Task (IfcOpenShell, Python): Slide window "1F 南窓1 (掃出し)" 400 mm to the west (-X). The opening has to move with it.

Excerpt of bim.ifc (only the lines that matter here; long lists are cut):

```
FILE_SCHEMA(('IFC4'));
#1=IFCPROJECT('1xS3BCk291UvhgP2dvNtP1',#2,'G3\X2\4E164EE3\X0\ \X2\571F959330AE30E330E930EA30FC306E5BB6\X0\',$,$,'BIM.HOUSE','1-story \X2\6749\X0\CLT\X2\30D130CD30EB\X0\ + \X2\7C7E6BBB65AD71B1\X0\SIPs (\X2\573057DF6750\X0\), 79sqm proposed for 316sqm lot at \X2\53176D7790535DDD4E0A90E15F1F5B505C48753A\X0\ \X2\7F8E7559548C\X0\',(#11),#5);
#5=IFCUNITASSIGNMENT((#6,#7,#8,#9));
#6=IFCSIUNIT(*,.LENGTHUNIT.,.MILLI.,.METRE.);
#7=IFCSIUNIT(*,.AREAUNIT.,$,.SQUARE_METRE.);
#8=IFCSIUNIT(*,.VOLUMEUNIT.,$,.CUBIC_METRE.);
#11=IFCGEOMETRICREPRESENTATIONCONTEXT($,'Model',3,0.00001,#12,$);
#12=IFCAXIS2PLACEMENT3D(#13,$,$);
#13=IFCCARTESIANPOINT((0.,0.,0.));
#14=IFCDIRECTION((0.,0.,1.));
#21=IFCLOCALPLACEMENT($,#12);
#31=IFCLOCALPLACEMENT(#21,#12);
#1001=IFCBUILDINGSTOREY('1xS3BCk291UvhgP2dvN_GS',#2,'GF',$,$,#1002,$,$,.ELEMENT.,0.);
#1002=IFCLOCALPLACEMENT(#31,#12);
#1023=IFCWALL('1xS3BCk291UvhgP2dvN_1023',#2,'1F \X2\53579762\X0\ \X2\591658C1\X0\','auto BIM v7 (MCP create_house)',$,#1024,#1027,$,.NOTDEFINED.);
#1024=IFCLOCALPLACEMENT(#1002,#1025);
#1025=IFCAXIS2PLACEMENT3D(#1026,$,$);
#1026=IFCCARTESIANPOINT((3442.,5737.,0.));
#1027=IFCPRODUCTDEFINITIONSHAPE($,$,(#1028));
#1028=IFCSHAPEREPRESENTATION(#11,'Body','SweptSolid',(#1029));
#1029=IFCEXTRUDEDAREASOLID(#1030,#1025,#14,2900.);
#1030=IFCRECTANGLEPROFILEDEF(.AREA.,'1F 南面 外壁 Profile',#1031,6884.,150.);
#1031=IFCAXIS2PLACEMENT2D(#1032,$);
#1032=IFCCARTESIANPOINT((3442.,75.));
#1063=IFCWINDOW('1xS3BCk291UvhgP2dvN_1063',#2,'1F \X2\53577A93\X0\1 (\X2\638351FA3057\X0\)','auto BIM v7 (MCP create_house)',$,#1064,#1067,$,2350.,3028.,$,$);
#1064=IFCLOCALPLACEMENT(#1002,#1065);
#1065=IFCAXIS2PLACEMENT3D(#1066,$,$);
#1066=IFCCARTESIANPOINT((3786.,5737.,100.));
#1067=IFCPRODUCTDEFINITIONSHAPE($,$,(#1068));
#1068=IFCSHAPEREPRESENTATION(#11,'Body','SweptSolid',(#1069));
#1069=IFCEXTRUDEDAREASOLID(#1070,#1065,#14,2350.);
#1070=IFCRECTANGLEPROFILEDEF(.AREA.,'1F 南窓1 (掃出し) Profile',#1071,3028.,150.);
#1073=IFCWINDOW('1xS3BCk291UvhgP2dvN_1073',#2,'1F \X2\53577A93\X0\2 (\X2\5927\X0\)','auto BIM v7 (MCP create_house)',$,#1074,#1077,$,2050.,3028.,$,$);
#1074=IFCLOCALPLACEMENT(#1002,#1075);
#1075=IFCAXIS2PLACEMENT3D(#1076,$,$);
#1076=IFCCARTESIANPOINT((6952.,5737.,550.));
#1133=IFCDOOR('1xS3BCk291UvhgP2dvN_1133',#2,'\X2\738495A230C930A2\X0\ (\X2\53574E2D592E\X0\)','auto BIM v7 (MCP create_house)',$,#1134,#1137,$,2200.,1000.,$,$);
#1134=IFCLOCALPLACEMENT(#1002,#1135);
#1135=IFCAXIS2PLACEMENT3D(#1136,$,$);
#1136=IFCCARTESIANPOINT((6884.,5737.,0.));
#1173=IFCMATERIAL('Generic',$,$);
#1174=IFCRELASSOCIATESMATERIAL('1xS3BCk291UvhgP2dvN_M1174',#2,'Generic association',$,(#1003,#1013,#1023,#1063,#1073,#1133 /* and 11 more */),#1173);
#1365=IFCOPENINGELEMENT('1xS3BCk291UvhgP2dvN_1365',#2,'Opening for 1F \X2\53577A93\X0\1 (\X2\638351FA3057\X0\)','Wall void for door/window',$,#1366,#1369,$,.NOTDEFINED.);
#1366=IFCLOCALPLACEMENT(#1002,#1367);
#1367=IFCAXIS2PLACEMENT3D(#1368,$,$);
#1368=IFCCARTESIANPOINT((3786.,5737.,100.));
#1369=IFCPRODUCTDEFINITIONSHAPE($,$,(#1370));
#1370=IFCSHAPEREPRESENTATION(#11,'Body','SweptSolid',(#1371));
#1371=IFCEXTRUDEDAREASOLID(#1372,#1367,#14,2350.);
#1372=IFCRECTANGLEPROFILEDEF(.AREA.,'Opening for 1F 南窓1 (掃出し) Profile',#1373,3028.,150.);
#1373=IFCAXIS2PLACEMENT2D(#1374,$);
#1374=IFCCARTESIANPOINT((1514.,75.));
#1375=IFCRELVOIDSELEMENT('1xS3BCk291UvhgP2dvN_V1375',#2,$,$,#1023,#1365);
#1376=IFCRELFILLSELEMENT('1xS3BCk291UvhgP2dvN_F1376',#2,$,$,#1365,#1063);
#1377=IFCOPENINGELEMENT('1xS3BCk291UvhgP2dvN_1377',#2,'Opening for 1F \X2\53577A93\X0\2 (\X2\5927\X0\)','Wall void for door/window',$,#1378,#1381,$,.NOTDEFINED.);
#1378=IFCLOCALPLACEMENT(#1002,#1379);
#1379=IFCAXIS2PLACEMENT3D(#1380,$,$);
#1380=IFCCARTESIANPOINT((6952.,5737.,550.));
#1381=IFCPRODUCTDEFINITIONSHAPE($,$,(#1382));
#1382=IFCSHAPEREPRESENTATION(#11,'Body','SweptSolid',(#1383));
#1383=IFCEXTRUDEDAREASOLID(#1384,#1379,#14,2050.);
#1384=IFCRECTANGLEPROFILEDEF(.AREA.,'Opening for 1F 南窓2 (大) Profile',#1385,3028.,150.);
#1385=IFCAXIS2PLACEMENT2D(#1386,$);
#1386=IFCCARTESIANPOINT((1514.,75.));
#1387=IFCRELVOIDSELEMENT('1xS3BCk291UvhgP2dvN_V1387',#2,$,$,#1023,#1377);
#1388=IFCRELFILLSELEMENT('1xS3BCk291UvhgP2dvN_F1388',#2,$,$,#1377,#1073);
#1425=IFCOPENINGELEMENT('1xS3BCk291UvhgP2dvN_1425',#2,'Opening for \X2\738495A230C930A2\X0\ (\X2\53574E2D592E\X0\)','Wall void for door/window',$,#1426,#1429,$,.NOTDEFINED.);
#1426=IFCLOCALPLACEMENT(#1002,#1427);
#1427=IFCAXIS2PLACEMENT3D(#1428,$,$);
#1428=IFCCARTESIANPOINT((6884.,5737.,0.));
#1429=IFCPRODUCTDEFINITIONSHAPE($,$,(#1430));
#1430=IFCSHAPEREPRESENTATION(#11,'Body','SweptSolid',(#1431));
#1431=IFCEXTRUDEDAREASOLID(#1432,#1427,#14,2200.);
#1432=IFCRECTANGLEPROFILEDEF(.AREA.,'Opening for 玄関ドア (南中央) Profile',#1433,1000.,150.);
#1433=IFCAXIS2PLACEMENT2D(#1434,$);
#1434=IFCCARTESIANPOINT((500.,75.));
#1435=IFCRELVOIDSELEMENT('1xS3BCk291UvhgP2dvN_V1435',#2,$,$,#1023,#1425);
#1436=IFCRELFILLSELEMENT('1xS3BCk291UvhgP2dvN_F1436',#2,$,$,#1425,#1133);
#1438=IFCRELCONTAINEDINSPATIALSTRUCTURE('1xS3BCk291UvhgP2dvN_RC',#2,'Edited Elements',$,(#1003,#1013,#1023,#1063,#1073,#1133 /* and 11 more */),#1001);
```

```python
import ifcopenshell
import ifcopenshell.api.geometry
import ifcopenshell.util.placement
import ifcopenshell.util.unit

model = ifcopenshell.open("bim.ifc")
unit_scale = ifcopenshell.util.unit.calculate_unit_scale(model)

window = model.by_guid("1xS3BCk291UvhgP2dvN_1063")
opening = window.FillsVoids[0].RelatingOpeningElement
wall = opening.VoidsElements[0].RelatingBuildingElement

wall_matrix = ifcopenshell.util.placement.get_local_placement(wall.ObjectPlacement)
shift = wall_matrix[:3, 0] * -0.4 / unit_scale
before = ifcopenshell.util.placement.get_local_placement(window.ObjectPlacement)[:3, 3].copy()

# The window is not placed relative to its opening, so move both.
for product in (opening, window):
    matrix = ifcopenshell.util.placement.get_local_placement(product.ObjectPlacement)
    matrix[:3, 3] += shift
    ifcopenshell.api.geometry.edit_object_placement(model, product=product, matrix=matrix, is_si=False)

after = ifcopenshell.util.placement.get_local_placement(window.ObjectPlacement)[:3, 3]
print("window moved by", (after - before).round(3) + 0.0)

model.write("bim_v2.ifc")
```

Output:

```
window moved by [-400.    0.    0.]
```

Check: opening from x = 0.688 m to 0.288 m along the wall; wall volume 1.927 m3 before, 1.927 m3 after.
